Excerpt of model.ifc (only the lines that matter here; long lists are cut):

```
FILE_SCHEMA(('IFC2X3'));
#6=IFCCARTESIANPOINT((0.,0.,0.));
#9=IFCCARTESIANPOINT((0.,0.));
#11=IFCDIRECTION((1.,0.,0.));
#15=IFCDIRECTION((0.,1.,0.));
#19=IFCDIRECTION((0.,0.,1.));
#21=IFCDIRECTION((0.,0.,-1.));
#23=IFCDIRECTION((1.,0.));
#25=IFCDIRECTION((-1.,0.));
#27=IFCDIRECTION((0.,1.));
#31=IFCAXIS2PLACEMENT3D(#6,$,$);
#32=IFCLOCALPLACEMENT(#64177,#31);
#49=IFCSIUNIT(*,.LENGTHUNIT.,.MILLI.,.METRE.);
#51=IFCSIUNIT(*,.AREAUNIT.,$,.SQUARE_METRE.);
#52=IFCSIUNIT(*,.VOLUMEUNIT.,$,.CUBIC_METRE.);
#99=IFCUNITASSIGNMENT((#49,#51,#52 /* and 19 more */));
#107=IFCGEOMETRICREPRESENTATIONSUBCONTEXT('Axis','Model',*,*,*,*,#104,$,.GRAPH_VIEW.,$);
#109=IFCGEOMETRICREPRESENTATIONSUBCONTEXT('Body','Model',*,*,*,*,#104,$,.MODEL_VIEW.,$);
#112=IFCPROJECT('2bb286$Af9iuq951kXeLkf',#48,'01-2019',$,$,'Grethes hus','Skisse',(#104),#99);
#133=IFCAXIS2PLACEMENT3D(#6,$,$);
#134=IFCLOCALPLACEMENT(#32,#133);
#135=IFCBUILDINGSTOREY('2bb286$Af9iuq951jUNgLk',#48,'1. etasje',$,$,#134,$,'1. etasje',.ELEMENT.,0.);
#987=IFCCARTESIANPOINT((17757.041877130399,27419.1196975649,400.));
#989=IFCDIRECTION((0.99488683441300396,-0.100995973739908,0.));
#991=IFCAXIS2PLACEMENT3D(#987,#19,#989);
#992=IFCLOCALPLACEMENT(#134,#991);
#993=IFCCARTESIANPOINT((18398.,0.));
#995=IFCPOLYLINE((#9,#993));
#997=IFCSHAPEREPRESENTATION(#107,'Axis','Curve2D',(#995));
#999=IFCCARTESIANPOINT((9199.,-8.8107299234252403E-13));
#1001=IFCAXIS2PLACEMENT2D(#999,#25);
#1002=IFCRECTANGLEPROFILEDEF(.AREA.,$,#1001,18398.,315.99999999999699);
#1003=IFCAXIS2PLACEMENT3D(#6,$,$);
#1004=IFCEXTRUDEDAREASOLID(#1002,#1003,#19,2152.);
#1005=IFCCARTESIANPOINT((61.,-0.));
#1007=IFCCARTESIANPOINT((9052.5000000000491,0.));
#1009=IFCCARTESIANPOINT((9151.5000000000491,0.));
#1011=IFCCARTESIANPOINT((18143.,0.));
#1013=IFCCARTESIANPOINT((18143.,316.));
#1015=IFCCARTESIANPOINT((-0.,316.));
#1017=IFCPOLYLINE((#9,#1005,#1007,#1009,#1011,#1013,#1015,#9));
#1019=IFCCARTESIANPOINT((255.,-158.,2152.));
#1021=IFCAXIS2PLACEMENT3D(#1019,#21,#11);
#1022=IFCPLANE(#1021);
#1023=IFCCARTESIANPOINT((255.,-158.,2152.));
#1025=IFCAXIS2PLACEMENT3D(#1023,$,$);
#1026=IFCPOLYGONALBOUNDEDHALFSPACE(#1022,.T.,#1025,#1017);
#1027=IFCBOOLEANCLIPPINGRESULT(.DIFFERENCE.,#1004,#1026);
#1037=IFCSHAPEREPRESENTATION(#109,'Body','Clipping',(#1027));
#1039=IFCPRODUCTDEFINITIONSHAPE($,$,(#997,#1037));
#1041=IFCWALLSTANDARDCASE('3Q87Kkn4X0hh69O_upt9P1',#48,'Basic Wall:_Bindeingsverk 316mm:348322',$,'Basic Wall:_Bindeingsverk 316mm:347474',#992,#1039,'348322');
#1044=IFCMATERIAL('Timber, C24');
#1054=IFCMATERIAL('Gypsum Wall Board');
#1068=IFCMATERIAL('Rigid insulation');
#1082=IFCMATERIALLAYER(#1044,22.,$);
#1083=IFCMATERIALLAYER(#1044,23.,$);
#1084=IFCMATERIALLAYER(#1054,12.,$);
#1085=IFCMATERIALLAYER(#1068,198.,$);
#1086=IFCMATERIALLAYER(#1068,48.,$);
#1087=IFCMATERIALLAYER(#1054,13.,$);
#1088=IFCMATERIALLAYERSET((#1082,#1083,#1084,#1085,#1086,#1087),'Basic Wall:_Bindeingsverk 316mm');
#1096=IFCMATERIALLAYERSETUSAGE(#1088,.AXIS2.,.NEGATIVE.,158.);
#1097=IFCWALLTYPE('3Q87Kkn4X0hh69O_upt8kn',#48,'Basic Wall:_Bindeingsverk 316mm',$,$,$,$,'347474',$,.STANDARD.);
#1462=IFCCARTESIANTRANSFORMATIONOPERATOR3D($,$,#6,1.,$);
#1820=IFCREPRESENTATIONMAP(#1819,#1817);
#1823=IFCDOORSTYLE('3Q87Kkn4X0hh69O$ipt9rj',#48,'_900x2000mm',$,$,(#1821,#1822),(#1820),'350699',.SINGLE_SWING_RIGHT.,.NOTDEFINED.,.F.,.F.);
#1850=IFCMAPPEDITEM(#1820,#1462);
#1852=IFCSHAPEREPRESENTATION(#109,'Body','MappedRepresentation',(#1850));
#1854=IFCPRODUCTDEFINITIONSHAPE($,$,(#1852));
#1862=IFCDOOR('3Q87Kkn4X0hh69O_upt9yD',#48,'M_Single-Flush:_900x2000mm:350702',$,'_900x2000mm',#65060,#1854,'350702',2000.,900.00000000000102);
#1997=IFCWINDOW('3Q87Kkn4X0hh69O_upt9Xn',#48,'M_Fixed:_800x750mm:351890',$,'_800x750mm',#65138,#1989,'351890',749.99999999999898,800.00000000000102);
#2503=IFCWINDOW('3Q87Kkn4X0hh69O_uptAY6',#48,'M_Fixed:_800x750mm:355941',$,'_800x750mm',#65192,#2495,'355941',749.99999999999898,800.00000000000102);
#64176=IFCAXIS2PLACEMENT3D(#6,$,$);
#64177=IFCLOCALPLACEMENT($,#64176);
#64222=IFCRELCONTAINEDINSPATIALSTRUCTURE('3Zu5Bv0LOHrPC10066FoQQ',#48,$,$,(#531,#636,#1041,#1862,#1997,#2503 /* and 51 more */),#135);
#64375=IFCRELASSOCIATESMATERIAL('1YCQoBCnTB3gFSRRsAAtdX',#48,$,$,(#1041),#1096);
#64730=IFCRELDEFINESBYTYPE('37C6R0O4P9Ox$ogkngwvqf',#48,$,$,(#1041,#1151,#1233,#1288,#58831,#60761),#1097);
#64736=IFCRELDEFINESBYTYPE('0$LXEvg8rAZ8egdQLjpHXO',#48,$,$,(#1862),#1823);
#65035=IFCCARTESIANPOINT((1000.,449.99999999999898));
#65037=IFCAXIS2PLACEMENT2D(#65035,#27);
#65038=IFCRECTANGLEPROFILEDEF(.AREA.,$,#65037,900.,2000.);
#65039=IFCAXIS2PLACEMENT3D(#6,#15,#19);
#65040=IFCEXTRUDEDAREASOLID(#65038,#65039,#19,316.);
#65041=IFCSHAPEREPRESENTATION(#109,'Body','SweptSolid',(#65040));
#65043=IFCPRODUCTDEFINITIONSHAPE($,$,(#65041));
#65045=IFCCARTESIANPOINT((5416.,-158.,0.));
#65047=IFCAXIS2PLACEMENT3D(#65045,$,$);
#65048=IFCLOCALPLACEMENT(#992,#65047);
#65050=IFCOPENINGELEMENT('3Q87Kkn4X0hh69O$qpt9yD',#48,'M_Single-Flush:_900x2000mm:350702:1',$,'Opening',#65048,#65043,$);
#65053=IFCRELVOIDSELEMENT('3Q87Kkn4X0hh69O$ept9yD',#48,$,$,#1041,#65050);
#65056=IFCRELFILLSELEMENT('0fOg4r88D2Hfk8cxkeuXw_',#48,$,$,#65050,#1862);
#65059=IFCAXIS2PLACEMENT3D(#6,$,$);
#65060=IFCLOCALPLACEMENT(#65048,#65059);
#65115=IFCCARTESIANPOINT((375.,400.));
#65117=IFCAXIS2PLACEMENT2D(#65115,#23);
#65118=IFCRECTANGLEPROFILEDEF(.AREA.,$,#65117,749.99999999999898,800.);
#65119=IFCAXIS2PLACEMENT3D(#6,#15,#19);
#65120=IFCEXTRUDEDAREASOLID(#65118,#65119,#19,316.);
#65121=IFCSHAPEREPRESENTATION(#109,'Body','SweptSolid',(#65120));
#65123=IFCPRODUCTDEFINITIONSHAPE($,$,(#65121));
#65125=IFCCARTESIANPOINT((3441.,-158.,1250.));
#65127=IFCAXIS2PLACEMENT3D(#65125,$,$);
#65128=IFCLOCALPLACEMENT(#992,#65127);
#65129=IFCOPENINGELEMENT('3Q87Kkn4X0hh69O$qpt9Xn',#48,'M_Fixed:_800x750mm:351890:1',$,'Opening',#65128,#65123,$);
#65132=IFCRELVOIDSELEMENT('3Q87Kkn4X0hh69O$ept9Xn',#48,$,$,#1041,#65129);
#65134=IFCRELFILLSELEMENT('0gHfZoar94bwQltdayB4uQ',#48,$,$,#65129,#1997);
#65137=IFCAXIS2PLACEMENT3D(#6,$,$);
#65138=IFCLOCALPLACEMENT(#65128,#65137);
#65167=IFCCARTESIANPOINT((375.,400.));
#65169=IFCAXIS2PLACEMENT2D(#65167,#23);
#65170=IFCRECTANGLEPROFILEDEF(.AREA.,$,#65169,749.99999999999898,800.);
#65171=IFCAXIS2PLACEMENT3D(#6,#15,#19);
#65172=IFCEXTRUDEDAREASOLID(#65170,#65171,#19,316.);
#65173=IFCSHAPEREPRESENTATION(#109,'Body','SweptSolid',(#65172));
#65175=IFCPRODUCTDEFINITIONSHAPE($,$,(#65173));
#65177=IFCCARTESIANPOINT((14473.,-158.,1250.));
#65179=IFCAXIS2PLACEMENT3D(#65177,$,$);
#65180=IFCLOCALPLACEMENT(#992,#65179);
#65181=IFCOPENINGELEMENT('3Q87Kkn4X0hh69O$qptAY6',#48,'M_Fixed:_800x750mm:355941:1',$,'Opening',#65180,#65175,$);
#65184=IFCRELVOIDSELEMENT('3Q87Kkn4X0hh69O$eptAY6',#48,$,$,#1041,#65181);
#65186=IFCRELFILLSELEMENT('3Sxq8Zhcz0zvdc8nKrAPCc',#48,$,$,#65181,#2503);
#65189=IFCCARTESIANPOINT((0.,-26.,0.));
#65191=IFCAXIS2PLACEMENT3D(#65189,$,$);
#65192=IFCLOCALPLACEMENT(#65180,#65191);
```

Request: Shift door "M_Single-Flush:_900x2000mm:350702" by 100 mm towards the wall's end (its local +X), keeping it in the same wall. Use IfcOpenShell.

```python
import ifcopenshell
import ifcopenshell.api.geometry
import ifcopenshell.util.placement
import ifcopenshell.util.unit

model = ifcopenshell.open("model.ifc")
unit_scale = ifcopenshell.util.unit.calculate_unit_scale(model)

door = model.by_guid("3Q87Kkn4X0hh69O_upt9yD")
opening = door.FillsVoids[0].RelatingOpeningElement
wall = opening.VoidsElements[0].RelatingBuildingElement

wall_matrix = ifcopenshell.util.placement.get_local_placement(wall.ObjectPlacement)
shift = wall_matrix[:3, 0] * 0.1 / unit_scale
before = ifcopenshell.util.placement.get_local_placement(door.ObjectPlacement)[:3, 3].copy()

# The door is placed relative to its opening, so it follows when the opening moves.
matrix = ifcopenshell.util.placement.get_local_placement(opening.ObjectPlacement)
matrix[:3, 3] += shift
ifcopenshell.api.geometry.edit_object_placement(
    model, product=opening, matrix=matrix, is_si=False, should_transform_children=True
)

after = ifcopenshell.util.placement.get_local_placement(door.ObjectPlacement)[:3, 3]
print("door moved by", (after - before).round(3) + 0.0)

model.write("model_rev.ifc")
```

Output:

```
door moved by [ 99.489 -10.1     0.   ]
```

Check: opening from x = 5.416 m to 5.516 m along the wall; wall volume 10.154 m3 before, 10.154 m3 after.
